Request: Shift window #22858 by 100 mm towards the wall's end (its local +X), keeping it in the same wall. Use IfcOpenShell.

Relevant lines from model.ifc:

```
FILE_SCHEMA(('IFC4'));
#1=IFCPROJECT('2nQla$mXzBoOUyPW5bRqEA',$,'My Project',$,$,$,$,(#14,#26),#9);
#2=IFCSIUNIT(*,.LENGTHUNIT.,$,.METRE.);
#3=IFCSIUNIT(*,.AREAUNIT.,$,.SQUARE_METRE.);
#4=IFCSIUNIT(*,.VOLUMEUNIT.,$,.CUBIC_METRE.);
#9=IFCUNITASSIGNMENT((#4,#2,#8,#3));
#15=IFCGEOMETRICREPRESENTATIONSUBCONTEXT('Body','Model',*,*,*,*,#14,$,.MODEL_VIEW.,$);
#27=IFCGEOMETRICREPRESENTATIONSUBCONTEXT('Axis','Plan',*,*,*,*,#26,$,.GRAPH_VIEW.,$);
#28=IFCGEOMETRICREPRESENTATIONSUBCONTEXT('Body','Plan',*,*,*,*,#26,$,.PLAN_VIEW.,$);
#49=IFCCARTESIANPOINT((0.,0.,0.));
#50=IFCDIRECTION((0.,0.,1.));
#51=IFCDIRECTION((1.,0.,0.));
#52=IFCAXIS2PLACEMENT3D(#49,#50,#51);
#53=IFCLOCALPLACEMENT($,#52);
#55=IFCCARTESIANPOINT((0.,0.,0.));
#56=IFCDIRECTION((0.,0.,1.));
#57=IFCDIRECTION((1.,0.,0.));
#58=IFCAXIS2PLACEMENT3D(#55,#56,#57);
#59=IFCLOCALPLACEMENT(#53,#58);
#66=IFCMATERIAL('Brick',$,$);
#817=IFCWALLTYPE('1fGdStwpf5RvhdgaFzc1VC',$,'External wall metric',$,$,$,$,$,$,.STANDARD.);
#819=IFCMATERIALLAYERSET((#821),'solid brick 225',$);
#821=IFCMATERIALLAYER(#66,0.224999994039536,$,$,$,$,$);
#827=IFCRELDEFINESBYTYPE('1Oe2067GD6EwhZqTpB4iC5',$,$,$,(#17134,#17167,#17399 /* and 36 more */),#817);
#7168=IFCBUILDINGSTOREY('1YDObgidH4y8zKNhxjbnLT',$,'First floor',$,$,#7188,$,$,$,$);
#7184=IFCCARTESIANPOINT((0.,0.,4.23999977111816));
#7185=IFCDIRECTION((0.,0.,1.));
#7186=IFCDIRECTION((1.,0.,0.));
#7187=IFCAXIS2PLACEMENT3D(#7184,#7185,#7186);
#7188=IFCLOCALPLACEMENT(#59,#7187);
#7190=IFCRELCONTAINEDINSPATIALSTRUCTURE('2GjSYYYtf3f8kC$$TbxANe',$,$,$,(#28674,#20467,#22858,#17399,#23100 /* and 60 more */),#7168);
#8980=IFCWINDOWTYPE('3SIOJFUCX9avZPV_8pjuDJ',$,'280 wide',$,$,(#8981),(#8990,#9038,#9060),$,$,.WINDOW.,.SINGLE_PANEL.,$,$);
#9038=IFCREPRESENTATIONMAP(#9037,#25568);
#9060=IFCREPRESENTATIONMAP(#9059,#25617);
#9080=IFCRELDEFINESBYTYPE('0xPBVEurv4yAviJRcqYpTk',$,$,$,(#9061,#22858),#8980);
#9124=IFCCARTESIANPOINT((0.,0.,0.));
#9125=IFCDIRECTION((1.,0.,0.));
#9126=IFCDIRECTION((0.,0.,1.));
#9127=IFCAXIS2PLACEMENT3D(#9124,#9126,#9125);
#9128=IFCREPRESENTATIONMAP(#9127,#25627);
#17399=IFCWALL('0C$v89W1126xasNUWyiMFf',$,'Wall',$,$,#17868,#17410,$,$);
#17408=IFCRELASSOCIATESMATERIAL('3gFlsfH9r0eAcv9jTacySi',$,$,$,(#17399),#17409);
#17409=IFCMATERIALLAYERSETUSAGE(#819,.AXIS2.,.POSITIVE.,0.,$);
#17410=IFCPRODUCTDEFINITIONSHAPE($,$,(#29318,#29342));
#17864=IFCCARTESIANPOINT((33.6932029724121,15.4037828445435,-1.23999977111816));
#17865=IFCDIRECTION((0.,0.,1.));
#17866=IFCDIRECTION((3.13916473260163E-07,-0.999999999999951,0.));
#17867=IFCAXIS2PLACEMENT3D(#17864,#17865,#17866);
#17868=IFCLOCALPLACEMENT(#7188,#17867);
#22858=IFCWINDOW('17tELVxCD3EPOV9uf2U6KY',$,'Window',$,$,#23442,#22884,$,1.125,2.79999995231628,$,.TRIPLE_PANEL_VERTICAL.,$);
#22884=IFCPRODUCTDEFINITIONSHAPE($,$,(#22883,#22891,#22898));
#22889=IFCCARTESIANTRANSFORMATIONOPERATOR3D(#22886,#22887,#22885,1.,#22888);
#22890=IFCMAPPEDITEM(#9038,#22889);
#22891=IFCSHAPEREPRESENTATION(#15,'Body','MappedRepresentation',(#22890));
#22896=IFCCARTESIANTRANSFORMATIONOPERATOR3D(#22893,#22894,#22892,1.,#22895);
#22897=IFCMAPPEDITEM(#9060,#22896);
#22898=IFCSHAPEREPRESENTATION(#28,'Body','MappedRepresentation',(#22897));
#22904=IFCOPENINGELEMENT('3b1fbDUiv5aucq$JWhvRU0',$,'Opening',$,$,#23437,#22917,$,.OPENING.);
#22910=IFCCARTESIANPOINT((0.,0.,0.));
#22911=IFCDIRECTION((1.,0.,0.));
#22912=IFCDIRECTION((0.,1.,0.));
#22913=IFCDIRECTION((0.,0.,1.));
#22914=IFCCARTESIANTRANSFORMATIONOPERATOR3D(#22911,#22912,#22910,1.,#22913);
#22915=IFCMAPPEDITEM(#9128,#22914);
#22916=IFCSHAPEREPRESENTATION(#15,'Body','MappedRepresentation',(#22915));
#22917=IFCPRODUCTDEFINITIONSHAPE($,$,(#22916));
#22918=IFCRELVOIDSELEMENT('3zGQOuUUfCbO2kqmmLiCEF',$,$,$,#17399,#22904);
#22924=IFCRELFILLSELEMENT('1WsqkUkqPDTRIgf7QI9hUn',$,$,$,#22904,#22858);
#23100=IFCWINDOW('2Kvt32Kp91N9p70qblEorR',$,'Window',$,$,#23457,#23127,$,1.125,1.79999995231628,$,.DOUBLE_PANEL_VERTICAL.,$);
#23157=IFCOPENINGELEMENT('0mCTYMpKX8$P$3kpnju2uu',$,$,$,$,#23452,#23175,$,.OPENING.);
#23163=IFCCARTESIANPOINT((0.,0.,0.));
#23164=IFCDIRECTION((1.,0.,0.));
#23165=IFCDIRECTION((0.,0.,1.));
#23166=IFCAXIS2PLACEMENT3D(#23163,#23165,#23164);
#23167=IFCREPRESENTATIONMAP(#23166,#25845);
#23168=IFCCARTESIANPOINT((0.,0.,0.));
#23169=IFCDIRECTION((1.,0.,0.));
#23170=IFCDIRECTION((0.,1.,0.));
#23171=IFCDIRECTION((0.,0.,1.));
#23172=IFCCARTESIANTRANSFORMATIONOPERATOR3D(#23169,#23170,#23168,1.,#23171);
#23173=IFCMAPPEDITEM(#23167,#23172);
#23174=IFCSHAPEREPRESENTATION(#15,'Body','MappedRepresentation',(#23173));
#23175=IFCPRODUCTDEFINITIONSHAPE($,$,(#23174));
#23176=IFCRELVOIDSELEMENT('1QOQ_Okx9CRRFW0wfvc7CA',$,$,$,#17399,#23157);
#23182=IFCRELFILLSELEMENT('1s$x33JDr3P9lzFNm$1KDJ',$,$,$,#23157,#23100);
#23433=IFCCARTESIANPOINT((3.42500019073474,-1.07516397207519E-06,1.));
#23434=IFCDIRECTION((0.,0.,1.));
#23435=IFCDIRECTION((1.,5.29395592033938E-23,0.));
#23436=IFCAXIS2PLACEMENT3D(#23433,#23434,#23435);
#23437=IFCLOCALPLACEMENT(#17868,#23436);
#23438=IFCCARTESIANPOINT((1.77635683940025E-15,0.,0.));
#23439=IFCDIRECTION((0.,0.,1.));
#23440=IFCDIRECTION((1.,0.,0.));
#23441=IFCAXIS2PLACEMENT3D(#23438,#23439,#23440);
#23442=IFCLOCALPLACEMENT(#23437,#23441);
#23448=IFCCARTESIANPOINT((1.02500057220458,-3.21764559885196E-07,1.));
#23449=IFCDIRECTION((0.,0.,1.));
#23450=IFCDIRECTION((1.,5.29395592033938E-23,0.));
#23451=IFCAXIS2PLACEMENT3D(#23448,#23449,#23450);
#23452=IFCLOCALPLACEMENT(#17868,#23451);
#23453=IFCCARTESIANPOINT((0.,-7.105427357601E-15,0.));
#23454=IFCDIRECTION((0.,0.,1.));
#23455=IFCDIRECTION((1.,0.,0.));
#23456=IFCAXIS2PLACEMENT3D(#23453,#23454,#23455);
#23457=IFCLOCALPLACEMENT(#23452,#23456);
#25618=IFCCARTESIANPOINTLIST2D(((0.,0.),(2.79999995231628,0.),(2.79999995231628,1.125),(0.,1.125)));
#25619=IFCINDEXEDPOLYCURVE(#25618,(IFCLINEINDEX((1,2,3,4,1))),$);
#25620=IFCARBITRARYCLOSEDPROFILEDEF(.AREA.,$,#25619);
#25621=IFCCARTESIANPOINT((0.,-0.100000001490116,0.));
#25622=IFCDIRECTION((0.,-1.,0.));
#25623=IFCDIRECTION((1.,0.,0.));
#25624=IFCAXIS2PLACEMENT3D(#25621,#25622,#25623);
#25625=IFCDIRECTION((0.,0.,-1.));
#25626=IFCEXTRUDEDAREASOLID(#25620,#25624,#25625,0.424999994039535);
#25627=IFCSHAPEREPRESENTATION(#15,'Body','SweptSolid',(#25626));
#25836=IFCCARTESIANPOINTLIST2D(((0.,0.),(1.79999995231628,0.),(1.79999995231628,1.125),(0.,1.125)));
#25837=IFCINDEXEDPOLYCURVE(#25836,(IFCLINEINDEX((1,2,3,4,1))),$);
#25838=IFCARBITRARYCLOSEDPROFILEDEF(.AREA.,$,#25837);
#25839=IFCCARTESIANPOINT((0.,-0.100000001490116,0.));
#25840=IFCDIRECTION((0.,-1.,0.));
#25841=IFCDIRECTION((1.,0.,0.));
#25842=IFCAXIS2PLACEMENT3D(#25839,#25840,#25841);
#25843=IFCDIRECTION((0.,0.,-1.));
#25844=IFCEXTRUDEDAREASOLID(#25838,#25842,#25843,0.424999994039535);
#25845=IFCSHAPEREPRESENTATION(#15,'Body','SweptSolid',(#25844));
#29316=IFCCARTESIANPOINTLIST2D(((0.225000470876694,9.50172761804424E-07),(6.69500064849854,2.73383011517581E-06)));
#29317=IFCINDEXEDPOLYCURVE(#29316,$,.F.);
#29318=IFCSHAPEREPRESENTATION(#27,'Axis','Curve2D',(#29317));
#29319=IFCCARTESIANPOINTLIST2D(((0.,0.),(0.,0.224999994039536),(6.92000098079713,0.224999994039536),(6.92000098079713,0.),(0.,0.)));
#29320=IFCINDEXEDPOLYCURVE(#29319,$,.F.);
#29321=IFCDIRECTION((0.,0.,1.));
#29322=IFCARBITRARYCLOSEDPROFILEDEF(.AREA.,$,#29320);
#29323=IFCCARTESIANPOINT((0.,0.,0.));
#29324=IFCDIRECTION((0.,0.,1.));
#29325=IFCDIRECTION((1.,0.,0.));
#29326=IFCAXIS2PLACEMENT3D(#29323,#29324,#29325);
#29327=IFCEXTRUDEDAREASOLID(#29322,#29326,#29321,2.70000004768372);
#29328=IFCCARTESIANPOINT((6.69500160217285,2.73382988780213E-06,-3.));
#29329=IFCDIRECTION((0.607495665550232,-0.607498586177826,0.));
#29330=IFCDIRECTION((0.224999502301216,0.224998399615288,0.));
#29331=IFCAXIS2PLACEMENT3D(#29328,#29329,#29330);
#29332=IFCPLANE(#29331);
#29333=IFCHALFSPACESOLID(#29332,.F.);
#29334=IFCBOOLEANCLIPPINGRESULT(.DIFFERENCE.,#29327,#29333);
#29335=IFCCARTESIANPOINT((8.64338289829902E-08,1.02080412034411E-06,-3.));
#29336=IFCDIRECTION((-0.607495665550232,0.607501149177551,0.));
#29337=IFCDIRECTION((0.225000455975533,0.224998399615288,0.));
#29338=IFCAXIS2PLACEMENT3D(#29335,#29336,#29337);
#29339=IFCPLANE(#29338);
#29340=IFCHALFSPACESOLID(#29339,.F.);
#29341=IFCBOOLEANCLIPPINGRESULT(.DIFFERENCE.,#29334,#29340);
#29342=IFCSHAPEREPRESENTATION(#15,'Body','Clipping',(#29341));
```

```python
import ifcopenshell
import ifcopenshell.api.geometry
import ifcopenshell.util.placement
import ifcopenshell.util.unit

model = ifcopenshell.open("model.ifc")
unit_scale = ifcopenshell.util.unit.calculate_unit_scale(model)

window = model.by_guid("17tELVxCD3EPOV9uf2U6KY")
opening = window.FillsVoids[0].RelatingOpeningElement
wall = opening.VoidsElements[0].RelatingBuildingElement

wall_matrix = ifcopenshell.util.placement.get_local_placement(wall.ObjectPlacement)
shift = wall_matrix[:3, 0] * 0.1 / unit_scale
before = ifcopenshell.util.placement.get_local_placement(window.ObjectPlacement)[:3, 3].copy()

# The window is placed relative to its opening, so it follows when the opening moves.
matrix = ifcopenshell.util.placement.get_local_placement(opening.ObjectPlacement)
matrix[:3, 3] += shift
ifcopenshell.api.geometry.edit_object_placement(
    model, product=opening, matrix=matrix, is_si=False, should_transform_children=True
)

after = ifcopenshell.util.placement.get_local_placement(window.ObjectPlacement)[:3, 3]
print("window moved by", (after - before).round(3) + 0.0)

model.write("model_edited.ifc")
```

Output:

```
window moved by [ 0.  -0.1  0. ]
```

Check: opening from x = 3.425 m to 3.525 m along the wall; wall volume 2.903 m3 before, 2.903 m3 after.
